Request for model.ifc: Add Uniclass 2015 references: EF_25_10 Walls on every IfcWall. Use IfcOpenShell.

First a look at what the model holds.

```python
import ifcopenshell

model = ifcopenshell.open("model.ifc")
print(model.schema)
print("classifications:", [c.Name for c in model.by_type("IfcClassification")])
for ifc_class in ("IfcDoor", "IfcRoof", "IfcStair", "IfcWall", "IfcWindow"):
    print(ifc_class, len(model.by_type(ifc_class)))
```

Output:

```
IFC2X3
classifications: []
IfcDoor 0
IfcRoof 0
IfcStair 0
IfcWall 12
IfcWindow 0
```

```python
import ifcopenshell
import ifcopenshell.api.classification

model = ifcopenshell.open("model.ifc")

# IFC2X3 requires Source and Edition and has no link from the project to the system.
system = model.create_entity("IfcClassification", Source="NBS", Edition="2015", Name="Uniclass 2015")

codes = {
    "IfcWall": ("EF_25_10", "Walls"),
}
for ifc_class, (code, name) in codes.items():
    products = model.by_type(ifc_class)
    ifcopenshell.api.classification.add_reference(
        model, products=products, classification=system, identification=code, name=name
    )
    print(code, len(products))

model.write("model_rev.ifc")
```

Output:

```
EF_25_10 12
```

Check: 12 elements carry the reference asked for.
